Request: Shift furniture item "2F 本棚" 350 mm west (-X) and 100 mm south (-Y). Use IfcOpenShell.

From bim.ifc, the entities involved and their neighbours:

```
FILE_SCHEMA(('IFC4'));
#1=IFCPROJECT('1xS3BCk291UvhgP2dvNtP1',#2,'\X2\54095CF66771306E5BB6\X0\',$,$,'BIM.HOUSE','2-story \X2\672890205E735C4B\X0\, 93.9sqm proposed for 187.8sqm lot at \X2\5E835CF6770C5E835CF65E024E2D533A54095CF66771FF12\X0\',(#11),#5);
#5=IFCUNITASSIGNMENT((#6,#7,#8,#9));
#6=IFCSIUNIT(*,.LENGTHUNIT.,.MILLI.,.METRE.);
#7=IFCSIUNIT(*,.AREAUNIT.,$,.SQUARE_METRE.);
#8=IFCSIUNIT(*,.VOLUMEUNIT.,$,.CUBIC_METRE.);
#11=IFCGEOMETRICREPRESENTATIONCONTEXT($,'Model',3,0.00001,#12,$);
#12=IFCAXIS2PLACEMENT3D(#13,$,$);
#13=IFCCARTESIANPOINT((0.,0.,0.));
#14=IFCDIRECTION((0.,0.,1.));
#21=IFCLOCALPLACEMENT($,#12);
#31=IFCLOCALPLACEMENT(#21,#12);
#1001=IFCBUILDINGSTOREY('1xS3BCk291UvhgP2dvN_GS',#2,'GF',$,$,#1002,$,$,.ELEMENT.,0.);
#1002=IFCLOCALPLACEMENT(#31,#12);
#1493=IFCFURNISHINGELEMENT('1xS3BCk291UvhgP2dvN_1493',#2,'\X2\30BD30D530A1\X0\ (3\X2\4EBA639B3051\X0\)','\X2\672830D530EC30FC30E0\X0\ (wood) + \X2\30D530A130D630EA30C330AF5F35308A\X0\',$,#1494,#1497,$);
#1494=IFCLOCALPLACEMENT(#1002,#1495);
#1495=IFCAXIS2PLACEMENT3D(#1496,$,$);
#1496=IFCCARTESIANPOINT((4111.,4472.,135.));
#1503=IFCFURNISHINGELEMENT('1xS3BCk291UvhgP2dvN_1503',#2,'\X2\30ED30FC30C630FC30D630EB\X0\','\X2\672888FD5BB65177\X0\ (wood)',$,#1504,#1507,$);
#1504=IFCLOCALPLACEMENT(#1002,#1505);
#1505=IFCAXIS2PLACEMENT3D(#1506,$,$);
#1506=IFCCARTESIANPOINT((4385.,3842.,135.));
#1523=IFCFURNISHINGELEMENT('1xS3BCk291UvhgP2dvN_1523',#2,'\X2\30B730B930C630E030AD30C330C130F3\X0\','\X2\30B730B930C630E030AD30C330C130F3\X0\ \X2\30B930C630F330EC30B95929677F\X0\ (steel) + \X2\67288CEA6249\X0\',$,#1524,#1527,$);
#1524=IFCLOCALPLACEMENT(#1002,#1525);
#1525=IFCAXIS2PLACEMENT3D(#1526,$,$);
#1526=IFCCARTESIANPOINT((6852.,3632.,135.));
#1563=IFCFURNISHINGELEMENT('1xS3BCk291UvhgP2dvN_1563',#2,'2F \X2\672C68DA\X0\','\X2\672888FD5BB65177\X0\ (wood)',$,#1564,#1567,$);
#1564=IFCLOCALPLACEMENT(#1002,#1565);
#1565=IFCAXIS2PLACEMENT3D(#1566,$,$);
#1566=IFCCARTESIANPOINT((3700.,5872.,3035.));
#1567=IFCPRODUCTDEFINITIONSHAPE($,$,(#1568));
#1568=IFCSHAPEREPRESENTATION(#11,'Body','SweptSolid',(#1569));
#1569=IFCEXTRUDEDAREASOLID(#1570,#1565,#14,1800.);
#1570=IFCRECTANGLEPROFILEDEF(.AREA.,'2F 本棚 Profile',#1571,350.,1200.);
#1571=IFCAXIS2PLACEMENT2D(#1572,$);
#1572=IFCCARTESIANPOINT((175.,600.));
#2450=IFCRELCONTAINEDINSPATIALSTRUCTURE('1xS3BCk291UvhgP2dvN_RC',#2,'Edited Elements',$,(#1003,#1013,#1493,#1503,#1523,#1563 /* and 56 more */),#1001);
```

```python
import ifcopenshell
import ifcopenshell.api.geometry
import ifcopenshell.util.placement

model = ifcopenshell.open("bim.ifc")

item = model.by_guid("1xS3BCk291UvhgP2dvN_1563")
matrix = ifcopenshell.util.placement.get_local_placement(item.ObjectPlacement)
matrix[0, 3] -= 350.0
matrix[1, 3] -= 100.0
ifcopenshell.api.geometry.edit_object_placement(model, product=item, matrix=matrix, is_si=False)

print(ifcopenshell.util.placement.get_local_placement(item.ObjectPlacement).round(3) + 0.0)

model.write("bim-out.ifc")
```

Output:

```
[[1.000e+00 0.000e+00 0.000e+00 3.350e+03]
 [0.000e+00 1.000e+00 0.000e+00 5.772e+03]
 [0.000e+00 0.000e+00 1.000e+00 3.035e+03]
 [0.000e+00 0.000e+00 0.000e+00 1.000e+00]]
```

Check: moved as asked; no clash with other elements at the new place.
